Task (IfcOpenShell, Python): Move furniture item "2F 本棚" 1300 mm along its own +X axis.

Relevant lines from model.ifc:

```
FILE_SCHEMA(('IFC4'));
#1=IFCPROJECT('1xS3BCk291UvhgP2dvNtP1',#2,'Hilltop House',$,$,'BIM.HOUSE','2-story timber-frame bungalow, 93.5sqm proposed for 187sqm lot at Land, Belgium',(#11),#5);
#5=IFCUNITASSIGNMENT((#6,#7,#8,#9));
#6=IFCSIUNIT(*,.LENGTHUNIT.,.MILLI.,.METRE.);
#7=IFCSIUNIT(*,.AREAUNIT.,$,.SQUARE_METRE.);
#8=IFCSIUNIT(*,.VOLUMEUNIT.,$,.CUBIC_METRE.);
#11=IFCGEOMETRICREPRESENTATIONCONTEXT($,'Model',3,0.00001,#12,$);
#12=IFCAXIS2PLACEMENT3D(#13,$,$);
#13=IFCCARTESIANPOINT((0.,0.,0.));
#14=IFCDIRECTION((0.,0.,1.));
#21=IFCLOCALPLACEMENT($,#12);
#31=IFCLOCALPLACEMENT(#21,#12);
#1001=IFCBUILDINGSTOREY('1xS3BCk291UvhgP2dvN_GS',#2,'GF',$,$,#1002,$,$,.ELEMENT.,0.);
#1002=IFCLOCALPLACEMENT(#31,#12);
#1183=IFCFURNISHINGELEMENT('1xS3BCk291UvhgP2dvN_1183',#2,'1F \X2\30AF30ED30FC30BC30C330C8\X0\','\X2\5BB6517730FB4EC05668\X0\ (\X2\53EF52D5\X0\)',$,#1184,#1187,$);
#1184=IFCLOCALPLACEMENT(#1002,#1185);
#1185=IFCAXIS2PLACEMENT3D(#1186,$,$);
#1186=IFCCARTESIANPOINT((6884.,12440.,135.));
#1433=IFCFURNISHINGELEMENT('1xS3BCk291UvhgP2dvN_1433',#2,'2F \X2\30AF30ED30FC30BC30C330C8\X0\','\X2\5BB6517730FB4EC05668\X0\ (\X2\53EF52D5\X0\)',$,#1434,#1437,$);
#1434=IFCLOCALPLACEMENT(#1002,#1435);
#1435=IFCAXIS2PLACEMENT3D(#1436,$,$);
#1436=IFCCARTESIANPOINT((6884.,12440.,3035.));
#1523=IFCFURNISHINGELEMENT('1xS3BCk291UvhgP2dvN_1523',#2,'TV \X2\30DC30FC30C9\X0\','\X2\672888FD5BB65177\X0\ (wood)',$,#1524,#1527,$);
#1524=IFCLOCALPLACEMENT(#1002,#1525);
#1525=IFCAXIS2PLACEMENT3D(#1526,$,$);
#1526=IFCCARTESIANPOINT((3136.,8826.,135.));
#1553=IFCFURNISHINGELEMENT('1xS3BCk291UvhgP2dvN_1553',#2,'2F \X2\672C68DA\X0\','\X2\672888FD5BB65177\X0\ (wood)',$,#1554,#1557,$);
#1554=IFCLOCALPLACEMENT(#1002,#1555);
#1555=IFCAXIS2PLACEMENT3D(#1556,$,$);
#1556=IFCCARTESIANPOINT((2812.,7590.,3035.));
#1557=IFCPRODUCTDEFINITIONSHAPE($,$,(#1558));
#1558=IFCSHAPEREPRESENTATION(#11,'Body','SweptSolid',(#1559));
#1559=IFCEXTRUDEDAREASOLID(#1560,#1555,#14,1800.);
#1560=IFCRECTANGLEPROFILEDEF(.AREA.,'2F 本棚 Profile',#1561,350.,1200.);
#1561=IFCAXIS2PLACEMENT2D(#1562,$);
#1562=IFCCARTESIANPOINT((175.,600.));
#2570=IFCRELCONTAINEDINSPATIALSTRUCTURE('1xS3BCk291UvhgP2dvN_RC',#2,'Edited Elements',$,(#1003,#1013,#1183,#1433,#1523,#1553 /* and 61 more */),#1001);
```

```python
import ifcopenshell
import ifcopenshell.api.geometry
import ifcopenshell.util.placement
import ifcopenshell.util.unit

model = ifcopenshell.open("model.ifc")
unit_scale = ifcopenshell.util.unit.calculate_unit_scale(model)

item = model.by_guid("1xS3BCk291UvhgP2dvN_1553")
matrix = ifcopenshell.util.placement.get_local_placement(item.ObjectPlacement)
matrix[:3, 3] += matrix[:3, 0] * 1.3 / unit_scale
ifcopenshell.api.geometry.edit_object_placement(model, product=item, matrix=matrix, is_si=False)

print(ifcopenshell.util.placement.get_local_placement(item.ObjectPlacement).round(3) + 0.0)

model.write("model-out.ifc")
```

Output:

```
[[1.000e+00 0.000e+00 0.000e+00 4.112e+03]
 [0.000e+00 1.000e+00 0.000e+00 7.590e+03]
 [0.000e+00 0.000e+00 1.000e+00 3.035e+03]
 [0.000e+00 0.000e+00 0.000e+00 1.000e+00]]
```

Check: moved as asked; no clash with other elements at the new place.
